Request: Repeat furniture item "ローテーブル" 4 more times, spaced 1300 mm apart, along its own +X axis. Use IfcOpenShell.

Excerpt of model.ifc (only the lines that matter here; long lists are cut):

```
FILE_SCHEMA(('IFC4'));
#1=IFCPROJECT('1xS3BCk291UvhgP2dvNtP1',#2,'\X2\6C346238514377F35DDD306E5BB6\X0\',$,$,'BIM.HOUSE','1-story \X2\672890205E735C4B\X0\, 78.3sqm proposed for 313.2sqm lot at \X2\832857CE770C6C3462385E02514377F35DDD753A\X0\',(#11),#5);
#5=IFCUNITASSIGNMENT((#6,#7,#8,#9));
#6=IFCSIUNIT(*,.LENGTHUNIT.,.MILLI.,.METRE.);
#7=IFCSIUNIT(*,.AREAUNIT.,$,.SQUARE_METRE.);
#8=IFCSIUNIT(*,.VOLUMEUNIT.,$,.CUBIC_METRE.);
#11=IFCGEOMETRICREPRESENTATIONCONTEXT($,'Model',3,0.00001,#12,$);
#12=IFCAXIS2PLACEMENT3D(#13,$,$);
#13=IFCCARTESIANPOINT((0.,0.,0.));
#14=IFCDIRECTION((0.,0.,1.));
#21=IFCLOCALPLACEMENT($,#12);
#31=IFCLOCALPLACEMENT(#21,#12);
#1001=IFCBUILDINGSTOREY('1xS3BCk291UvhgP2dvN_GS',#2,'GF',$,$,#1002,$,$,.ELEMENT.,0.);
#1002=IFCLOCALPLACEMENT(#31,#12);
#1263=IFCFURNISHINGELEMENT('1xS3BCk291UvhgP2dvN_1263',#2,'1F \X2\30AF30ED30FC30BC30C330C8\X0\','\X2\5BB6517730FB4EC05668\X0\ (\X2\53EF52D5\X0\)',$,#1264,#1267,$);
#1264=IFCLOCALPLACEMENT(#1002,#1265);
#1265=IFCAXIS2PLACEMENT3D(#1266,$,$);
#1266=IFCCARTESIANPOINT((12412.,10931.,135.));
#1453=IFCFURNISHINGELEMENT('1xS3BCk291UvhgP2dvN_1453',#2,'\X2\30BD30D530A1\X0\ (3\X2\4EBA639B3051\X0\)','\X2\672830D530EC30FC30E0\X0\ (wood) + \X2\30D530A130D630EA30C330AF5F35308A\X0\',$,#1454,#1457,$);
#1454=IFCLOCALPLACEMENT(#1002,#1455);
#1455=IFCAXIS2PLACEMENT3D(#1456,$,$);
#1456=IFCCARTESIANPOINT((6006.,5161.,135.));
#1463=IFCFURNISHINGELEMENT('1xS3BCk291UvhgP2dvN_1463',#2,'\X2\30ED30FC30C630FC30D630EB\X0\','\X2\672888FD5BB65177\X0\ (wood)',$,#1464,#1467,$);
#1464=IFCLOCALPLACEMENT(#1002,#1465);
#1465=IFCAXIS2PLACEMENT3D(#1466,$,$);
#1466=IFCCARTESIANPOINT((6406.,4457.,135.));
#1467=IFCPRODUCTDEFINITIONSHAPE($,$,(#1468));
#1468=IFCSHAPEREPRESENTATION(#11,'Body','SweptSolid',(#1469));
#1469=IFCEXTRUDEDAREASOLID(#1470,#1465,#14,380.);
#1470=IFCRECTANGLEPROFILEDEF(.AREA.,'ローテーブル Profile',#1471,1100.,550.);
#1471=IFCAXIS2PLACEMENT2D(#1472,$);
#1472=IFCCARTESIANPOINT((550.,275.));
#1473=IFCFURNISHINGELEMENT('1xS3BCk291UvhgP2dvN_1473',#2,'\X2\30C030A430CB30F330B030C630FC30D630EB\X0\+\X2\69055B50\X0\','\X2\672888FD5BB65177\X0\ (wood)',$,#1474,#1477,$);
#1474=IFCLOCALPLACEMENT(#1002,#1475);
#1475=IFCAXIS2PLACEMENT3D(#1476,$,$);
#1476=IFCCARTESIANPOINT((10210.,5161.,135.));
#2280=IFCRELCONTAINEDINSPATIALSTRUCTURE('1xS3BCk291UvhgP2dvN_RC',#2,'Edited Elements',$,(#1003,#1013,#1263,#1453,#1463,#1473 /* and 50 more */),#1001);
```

```python
import ifcopenshell
import ifcopenshell.api.geometry
import ifcopenshell.api.root
import ifcopenshell.util.element
import ifcopenshell.util.placement
import ifcopenshell.util.unit

model = ifcopenshell.open("model.ifc")
unit_scale = ifcopenshell.util.unit.calculate_unit_scale(model)


def reuse_history(source, copy):
    """copy_class also copies each property set's owner history, people and application; keep the originals."""
    for rel in copy.IsDefinedBy:
        if rel.is_a("IfcRelDefinesByProperties") and (history := rel.RelatingPropertyDefinition.OwnerHistory):
            rel.RelatingPropertyDefinition.OwnerHistory = source.OwnerHistory
            ifcopenshell.util.element.remove_deep2(model, history)


source = model.by_guid("1xS3BCk291UvhgP2dvN_1463")
base = ifcopenshell.util.placement.get_local_placement(source.ObjectPlacement)
step = base[:3, 0] * 1.3 / unit_scale

for i in range(1, 5):
    copy = ifcopenshell.api.root.copy_class(model, product=source)
    copy.Representation = ifcopenshell.util.element.copy_deep(
        model, source.Representation, exclude=["IfcGeometricRepresentationContext", "IfcRepresentationMap"]
    )
    reuse_history(source, copy)
    matrix = base.copy()
    matrix[:3, 3] += i * step
    print("added at", matrix[:3, 3].round(3) + 0.0)
    ifcopenshell.api.geometry.edit_object_placement(model, product=copy, matrix=matrix, is_si=False)

model.write("model-out.ifc")
```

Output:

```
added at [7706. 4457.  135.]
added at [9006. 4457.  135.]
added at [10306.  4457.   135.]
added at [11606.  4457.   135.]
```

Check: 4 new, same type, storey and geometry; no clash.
